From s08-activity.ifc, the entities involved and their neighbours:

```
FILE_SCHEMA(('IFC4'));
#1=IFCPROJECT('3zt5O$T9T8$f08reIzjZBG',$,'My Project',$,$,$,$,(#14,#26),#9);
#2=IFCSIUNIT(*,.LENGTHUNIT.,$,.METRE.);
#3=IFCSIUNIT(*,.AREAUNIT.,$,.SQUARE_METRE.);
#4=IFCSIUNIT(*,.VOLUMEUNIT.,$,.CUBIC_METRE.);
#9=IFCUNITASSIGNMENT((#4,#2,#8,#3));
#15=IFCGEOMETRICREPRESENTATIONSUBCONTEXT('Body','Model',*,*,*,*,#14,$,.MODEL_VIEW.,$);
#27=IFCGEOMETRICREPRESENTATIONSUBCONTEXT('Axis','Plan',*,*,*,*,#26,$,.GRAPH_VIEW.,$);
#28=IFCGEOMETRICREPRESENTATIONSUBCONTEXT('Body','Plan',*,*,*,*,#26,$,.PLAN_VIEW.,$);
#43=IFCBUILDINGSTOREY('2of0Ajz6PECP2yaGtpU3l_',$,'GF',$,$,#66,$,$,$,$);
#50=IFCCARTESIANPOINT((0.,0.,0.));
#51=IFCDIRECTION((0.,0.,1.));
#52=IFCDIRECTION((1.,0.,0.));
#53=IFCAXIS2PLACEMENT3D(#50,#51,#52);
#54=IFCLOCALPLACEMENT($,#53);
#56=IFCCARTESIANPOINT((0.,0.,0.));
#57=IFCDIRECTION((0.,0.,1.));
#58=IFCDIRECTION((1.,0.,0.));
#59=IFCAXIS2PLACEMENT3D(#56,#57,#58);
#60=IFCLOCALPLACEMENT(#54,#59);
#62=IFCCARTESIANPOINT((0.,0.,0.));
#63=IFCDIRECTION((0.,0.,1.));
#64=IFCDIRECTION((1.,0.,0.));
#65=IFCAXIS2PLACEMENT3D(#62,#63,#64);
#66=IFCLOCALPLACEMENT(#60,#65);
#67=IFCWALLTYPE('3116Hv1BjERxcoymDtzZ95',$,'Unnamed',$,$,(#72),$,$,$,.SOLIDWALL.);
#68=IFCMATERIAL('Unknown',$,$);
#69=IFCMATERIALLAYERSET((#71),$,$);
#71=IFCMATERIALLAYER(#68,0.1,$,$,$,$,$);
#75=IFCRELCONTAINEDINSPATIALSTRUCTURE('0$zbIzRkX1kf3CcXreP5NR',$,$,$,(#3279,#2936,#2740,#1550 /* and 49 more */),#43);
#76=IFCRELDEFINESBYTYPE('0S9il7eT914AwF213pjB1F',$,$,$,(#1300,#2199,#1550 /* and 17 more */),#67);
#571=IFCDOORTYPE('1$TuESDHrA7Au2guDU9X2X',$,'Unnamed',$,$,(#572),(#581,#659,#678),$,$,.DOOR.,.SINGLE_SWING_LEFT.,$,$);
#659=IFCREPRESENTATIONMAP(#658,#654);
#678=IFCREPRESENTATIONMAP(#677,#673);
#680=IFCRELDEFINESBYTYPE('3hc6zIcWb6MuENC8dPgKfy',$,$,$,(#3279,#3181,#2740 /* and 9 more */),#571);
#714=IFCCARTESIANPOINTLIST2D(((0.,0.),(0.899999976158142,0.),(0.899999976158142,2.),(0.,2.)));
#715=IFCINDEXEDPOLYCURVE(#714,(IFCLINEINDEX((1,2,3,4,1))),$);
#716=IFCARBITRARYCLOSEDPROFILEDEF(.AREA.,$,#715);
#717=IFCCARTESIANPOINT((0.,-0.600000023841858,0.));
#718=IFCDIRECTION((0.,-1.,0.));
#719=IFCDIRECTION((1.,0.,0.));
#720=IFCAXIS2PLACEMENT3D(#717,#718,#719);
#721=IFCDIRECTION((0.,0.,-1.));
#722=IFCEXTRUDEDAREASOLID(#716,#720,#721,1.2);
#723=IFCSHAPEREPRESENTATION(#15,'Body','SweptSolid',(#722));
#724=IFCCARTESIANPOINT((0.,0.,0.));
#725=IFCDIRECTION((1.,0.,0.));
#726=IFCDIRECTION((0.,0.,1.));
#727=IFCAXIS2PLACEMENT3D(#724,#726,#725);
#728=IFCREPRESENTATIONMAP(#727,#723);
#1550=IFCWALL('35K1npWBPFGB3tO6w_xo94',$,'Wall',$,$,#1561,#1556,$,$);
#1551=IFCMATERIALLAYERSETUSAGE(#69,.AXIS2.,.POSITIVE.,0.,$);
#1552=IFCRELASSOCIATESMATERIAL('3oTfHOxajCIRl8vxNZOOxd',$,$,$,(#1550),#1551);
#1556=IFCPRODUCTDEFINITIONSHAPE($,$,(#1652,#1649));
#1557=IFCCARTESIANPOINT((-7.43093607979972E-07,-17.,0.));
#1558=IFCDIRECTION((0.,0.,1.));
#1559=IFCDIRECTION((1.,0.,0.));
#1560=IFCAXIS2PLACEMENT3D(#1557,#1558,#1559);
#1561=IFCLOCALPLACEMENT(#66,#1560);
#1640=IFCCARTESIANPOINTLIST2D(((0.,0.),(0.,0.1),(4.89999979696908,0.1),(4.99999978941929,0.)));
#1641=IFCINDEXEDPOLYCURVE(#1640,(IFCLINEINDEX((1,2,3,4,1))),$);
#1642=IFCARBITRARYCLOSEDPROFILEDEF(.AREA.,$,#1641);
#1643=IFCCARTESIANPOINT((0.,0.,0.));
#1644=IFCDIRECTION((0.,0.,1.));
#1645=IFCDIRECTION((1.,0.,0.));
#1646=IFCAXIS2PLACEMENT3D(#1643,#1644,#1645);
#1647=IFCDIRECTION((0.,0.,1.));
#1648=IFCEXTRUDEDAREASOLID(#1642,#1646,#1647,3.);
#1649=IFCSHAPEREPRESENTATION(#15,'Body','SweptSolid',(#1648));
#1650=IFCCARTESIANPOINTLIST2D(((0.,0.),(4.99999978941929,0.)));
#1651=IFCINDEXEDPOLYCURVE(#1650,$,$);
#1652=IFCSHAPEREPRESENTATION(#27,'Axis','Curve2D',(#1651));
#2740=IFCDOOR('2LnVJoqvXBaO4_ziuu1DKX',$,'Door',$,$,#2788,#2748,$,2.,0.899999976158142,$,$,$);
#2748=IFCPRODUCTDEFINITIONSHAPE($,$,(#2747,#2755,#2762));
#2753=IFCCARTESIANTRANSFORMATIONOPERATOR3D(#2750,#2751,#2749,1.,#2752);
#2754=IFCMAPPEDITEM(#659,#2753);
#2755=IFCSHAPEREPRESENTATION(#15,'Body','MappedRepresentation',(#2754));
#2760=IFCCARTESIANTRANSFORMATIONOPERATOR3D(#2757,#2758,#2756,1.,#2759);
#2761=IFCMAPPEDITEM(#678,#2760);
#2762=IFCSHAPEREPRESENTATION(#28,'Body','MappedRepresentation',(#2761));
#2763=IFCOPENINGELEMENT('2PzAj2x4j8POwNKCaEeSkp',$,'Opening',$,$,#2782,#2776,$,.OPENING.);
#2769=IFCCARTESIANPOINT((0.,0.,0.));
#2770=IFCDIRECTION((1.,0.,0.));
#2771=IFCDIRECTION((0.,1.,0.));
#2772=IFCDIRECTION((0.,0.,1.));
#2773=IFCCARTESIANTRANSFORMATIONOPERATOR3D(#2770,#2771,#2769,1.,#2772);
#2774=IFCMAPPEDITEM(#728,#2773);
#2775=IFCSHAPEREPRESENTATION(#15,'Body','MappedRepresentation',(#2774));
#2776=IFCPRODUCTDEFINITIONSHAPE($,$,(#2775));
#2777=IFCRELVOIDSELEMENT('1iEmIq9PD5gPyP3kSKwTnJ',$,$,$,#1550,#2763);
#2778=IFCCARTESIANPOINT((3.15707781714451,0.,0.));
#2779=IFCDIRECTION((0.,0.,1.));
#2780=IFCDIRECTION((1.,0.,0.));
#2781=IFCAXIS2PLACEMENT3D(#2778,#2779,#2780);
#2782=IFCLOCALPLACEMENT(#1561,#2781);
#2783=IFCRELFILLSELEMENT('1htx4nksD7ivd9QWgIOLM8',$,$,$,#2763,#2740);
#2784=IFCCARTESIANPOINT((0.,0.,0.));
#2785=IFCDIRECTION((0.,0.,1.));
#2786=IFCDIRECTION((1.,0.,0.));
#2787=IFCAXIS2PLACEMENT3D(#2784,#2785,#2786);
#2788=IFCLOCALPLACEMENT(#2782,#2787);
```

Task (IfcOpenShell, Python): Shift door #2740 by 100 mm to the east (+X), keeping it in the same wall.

```python
import ifcopenshell
import ifcopenshell.api.geometry
import ifcopenshell.util.placement

model = ifcopenshell.open("s08-activity.ifc")

door = model.by_guid("2LnVJoqvXBaO4_ziuu1DKX")
opening = door.FillsVoids[0].RelatingOpeningElement
wall = opening.VoidsElements[0].RelatingBuildingElement

wall_matrix = ifcopenshell.util.placement.get_local_placement(wall.ObjectPlacement)
shift = wall_matrix[:3, 0] * 0.1
before = ifcopenshell.util.placement.get_local_placement(door.ObjectPlacement)[:3, 3].copy()

# The door is placed relative to its opening, so it follows when the opening moves.
matrix = ifcopenshell.util.placement.get_local_placement(opening.ObjectPlacement)
matrix[:3, 3] += shift
ifcopenshell.api.geometry.edit_object_placement(
    model, product=opening, matrix=matrix, is_si=False, should_transform_children=True
)

after = ifcopenshell.util.placement.get_local_placement(door.ObjectPlacement)[:3, 3]
print("door moved by", (after - before).round(3) + 0.0)

model.write("s08-activity_rev.ifc")
```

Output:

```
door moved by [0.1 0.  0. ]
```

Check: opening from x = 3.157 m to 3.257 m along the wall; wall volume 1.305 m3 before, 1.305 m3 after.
